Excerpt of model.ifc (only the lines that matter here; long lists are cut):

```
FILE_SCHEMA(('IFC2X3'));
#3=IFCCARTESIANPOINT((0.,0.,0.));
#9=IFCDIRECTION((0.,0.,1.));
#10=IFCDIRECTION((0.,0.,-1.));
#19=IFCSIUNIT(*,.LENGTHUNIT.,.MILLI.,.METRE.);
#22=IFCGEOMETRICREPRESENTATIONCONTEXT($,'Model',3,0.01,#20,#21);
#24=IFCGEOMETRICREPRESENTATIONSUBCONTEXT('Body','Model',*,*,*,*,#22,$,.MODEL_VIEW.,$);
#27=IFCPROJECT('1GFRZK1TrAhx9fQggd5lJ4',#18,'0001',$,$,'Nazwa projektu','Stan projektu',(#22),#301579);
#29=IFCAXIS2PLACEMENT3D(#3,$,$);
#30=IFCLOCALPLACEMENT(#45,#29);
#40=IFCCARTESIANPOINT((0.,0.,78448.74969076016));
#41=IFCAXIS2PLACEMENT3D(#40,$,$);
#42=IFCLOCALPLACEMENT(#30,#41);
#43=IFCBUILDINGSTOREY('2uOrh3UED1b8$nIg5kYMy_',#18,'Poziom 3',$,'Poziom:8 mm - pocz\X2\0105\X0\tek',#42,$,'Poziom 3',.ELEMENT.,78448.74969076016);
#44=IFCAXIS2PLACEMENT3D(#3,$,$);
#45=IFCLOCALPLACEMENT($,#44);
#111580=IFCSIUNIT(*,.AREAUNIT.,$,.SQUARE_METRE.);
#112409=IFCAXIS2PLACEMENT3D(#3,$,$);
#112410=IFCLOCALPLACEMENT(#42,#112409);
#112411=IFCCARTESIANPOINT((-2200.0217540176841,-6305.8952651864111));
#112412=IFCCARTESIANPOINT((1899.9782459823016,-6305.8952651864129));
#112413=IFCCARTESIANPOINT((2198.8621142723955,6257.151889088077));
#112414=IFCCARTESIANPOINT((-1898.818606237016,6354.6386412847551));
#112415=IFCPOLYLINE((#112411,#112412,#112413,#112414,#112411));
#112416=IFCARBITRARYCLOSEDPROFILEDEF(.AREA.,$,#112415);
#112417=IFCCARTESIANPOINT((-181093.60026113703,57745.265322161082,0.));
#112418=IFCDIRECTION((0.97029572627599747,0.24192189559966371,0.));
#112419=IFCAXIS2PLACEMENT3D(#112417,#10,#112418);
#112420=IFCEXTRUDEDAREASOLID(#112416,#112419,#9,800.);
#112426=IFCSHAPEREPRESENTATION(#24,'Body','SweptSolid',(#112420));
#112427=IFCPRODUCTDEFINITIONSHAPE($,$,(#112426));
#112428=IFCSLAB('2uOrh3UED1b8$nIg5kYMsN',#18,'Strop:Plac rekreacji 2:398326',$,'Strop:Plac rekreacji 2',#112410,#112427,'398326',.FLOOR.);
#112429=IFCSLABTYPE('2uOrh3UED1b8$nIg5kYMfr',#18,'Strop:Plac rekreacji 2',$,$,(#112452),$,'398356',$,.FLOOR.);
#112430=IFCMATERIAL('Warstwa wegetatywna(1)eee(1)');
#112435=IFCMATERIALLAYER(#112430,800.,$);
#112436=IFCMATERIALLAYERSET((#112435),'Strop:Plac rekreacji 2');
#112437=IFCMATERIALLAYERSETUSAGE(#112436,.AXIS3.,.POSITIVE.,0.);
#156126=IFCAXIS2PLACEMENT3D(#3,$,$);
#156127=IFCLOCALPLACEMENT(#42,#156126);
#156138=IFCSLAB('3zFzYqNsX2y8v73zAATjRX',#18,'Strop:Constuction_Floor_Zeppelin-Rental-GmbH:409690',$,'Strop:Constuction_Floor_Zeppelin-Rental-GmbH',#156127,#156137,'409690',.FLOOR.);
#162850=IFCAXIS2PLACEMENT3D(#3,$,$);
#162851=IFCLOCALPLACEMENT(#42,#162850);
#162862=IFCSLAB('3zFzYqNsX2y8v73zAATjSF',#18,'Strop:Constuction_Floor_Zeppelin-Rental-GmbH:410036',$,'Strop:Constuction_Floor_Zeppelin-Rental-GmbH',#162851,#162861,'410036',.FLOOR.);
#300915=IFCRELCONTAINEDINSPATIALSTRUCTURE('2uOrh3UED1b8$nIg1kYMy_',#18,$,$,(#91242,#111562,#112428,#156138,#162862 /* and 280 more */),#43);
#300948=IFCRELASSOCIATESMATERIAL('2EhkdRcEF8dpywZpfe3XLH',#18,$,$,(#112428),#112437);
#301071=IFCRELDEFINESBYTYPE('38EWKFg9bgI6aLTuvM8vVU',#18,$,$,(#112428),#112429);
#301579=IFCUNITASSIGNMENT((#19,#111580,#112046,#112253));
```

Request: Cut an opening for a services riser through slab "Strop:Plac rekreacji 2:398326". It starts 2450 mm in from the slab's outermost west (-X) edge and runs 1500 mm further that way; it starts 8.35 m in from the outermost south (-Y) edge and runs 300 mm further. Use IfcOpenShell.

```python
import numpy as np
import ifcopenshell
import ifcopenshell.api.feature
import ifcopenshell.api.geometry
import ifcopenshell.api.root
import ifcopenshell.geom
import ifcopenshell.util.placement
import ifcopenshell.util.representation
import ifcopenshell.util.shape
import ifcopenshell.util.unit

model = ifcopenshell.open("model.ifc")
unit_scale = ifcopenshell.util.unit.calculate_unit_scale(model)
settings = ifcopenshell.geom.settings()


def volume(element):
    """Net volume in cubic metres, openings subtracted."""
    shape = ifcopenshell.geom.create_shape(settings, element)
    return ifcopenshell.util.shape.get_volume(shape.geometry)


slab = model.by_guid("2uOrh3UED1b8$nIg5kYMsN")
before = volume(slab)

# Extent in the slab's own axes, in metres. The edges named are its -X and -Y sides.
slab_shape = ifcopenshell.geom.create_shape(settings, slab)
vertices = ifcopenshell.util.shape.get_vertices(slab_shape.geometry)
x_min, y_min, bottom = vertices.min(axis=0)
top = vertices[:, 2].max()

opening = ifcopenshell.api.root.create_entity(model, ifc_class="IfcOpeningElement", name="Services riser opening")
context = ifcopenshell.util.representation.get_context(model, "Model", "Body", "MODEL_VIEW")
width, depth = 1.5, 0.3
outline = [(0.0, 0.0), (width, 0.0), (width, depth), (0.0, depth), (0.0, 0.0)]
# Overshoot both faces by 50 mm so the cut is clean.
shape = ifcopenshell.api.geometry.add_slab_representation(
    model, context=context, depth=top - bottom + 0.1, polyline=outline
)
ifcopenshell.api.geometry.assign_representation(model, product=opening, representation=shape)

matrix = ifcopenshell.util.placement.get_local_placement(slab.ObjectPlacement)
matrix[:, 3] = matrix @ np.append(np.array([x_min + 2.45, y_min + 8.35, bottom - 0.05]) / unit_scale, 1.0)
ifcopenshell.api.geometry.edit_object_placement(model, product=opening, matrix=matrix, is_si=False)
ifcopenshell.api.feature.add_feature(model, feature=opening, element=slab)

after = volume(slab)

print(f"slab volume {before:.3f} -> {after:.3f} m3")

model.write("model_v2.ifc")
```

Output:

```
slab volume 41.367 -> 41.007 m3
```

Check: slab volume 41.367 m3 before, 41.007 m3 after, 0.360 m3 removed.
